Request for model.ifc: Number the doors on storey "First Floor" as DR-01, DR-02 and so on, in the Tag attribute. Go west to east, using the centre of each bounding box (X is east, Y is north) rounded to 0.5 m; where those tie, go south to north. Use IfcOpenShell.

First a look at what the model holds.

```python
import ifcopenshell
import ifcopenshell.util.element
import ifcopenshell.util.placement

model = ifcopenshell.open("model.ifc")
print(model.schema)
storey = next(s for s in model.by_type("IfcBuildingStorey") if s.Name == "First Floor")
doors = [e for e in ifcopenshell.util.element.get_decomposition(storey) if e.is_a("IfcDoor")]
for e in sorted(doors, key=lambda e: e.id()):
    origin = ifcopenshell.util.placement.get_local_placement(e.ObjectPlacement)[:3, 3]
    print(e.id(), e.Tag, e.Name, origin.round(2) + 0.0, sep=" | ")
```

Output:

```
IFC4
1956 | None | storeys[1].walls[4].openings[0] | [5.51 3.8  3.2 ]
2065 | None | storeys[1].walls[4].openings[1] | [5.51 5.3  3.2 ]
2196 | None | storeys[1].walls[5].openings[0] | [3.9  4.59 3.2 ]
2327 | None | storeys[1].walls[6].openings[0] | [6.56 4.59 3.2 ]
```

```python
import ifcopenshell
import ifcopenshell.geom
import ifcopenshell.util.element
import ifcopenshell.util.shape

model = ifcopenshell.open("model.ifc")
settings = ifcopenshell.geom.settings()
settings.set("use-world-coords", True)


def centre(element):
    shape = ifcopenshell.geom.create_shape(settings, element)
    return ifcopenshell.util.shape.get_bbox_centroid(shape.geometry)


storey = next(s for s in model.by_type("IfcBuildingStorey") if s.Name == "First Floor")
doors = [e for e in ifcopenshell.util.element.get_decomposition(storey) if e.is_a("IfcDoor")]

# Insertion points can sit at a corner or the storey origin, so sort by the geometry (in metres).
centres = {e: centre(e) for e in doors}
doors.sort(key=lambda e: (round(centres[e][0] / 0.5), centres[e][1]))

for i, e in enumerate(doors, start=1):
    number = f"DR-{i:02d}"
    e.Tag = number
    print(e.id(), number)

model.write("model_updated.ifc")
```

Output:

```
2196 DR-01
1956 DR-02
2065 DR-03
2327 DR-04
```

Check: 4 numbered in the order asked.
